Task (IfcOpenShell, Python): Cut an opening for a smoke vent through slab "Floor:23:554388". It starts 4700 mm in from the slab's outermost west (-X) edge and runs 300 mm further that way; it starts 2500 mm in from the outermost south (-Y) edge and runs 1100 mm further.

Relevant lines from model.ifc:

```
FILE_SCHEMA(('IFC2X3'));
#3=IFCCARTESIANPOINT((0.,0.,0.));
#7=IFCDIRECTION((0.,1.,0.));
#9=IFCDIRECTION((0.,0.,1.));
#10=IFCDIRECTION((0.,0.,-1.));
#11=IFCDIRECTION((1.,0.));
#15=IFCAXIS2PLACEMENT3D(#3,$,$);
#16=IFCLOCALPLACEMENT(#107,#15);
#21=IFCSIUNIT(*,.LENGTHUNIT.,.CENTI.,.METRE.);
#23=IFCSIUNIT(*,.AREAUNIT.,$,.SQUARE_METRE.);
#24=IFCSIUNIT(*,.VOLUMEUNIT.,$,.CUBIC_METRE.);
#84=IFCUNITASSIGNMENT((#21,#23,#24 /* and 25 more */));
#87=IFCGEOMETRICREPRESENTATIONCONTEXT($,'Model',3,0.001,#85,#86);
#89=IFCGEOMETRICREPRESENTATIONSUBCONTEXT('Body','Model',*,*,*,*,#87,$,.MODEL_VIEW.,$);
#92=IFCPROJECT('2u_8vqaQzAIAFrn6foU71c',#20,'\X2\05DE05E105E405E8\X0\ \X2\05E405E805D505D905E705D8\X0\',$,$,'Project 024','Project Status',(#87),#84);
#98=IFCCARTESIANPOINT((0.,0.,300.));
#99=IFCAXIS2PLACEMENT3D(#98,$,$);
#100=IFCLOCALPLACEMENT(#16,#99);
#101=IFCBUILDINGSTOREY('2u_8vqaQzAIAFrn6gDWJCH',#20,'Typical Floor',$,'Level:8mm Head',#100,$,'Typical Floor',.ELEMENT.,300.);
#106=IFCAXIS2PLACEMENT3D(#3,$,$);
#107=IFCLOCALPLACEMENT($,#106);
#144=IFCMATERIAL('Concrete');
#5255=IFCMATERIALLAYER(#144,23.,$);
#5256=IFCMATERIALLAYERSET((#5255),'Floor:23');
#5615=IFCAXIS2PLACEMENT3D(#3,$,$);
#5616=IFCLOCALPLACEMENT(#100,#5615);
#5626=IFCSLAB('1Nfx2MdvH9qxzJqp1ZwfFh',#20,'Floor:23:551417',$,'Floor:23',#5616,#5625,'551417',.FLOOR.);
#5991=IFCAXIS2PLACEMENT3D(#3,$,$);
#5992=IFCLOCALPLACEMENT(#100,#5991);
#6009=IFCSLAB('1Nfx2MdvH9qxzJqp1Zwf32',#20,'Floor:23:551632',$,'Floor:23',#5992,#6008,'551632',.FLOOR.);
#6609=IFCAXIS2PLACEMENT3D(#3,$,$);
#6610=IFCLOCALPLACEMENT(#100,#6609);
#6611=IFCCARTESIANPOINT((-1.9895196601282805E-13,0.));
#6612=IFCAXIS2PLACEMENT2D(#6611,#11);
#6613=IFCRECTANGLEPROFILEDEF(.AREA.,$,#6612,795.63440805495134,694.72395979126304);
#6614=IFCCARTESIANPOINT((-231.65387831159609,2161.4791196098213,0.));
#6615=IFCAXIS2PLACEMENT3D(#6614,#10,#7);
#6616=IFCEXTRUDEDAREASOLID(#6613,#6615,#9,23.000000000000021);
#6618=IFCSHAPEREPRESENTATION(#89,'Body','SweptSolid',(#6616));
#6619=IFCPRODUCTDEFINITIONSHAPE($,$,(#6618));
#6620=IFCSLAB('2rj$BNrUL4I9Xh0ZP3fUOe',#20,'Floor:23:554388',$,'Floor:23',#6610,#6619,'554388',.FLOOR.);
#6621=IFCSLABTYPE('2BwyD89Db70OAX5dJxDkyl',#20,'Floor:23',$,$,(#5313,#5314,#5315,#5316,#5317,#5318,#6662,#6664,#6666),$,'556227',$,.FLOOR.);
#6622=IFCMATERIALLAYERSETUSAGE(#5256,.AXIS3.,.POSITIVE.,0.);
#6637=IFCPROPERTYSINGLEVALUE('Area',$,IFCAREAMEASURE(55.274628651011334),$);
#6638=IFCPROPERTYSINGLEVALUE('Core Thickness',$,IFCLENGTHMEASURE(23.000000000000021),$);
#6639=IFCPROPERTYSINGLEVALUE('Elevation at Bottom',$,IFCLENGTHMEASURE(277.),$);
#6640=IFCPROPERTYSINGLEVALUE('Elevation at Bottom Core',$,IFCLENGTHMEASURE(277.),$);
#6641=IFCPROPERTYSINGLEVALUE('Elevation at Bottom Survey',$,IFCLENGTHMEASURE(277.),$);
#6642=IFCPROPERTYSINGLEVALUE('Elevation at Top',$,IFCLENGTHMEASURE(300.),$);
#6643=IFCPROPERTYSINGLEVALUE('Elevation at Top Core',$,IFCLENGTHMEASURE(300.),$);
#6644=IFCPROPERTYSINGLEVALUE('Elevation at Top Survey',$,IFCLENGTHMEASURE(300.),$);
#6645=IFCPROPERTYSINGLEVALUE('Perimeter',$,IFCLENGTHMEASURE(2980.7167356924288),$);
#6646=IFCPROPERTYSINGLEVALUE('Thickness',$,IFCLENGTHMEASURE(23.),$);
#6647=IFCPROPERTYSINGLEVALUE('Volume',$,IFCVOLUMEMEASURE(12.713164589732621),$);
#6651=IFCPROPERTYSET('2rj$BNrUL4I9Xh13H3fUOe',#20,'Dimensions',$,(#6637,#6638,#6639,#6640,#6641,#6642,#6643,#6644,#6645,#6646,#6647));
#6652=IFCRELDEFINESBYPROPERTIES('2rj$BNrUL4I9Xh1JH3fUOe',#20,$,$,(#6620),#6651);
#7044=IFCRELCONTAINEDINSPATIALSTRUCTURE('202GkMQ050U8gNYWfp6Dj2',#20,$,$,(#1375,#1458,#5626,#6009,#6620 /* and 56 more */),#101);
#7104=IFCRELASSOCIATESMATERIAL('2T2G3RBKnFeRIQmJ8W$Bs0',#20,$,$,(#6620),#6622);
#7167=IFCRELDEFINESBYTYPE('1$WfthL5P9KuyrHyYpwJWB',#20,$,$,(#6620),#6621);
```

```python
import numpy as np
import ifcopenshell
import ifcopenshell.api.feature
import ifcopenshell.api.geometry
import ifcopenshell.api.pset
import ifcopenshell.api.root
import ifcopenshell.geom
import ifcopenshell.util.element
import ifcopenshell.util.placement
import ifcopenshell.util.representation
import ifcopenshell.util.shape
import ifcopenshell.util.unit

model = ifcopenshell.open("model.ifc")
unit_scale = ifcopenshell.util.unit.calculate_unit_scale(model)
area_scale = ifcopenshell.util.unit.calculate_unit_scale(model, "AREAUNIT")
volume_scale = ifcopenshell.util.unit.calculate_unit_scale(model, "VOLUMEUNIT")
settings = ifcopenshell.geom.settings()


def volume(element):
    """Net volume in cubic metres, openings subtracted."""
    shape = ifcopenshell.geom.create_shape(settings, element)
    return ifcopenshell.util.shape.get_volume(shape.geometry)


slab = model.by_guid("2rj$BNrUL4I9Xh0ZP3fUOe")
before = volume(slab)

# Extent in the slab's own axes, in metres. The edges named are its -X and -Y sides.
slab_shape = ifcopenshell.geom.create_shape(settings, slab)
vertices = ifcopenshell.util.shape.get_vertices(slab_shape.geometry)
x_min, y_min, bottom = vertices.min(axis=0)
top = vertices[:, 2].max()

opening = ifcopenshell.api.root.create_entity(model, ifc_class="IfcOpeningElement", name="Smoke vent opening")
context = ifcopenshell.util.representation.get_context(model, "Model", "Body", "MODEL_VIEW")
width, depth = 0.3, 1.1
outline = [(0.0, 0.0), (width, 0.0), (width, depth), (0.0, depth), (0.0, 0.0)]
# Overshoot both faces by 50 mm so the cut is clean.
shape = ifcopenshell.api.geometry.add_slab_representation(
    model, context=context, depth=top - bottom + 0.1, polyline=outline
)
ifcopenshell.api.geometry.assign_representation(model, product=opening, representation=shape)

matrix = ifcopenshell.util.placement.get_local_placement(slab.ObjectPlacement)
matrix[:, 3] = matrix @ np.append(np.array([x_min + 4.7, y_min + 2.5, bottom - 0.05]) / unit_scale, 1.0)
ifcopenshell.api.geometry.edit_object_placement(model, product=opening, matrix=matrix, is_si=False)
ifcopenshell.api.feature.add_feature(model, feature=opening, element=slab)

after = volume(slab)

# Update the slab's stored quantities.
pset = model.by_id(ifcopenshell.util.element.get_pset(slab, "Dimensions", should_inherit=False)["id"])
ifcopenshell.api.pset.edit_pset(model, pset=pset, properties={
    "Area": model.create_entity("IfcAreaMeasure", after / (top - bottom) / area_scale),
    "Volume": model.create_entity("IfcVolumeMeasure", after / volume_scale),
})

print(f"slab volume {before:.3f} -> {after:.3f} m3")

model.write("model_rev.ifc")
```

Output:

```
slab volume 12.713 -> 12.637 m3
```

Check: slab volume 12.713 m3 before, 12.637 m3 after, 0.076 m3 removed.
